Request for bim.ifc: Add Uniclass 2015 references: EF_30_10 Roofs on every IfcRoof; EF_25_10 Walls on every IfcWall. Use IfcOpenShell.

First a look at what the model holds.

```python
import ifcopenshell

model = ifcopenshell.open("bim.ifc")
print(model.schema)
print("classifications:", [c.Name for c in model.by_type("IfcClassification")])
for ifc_class in ("IfcDoor", "IfcRoof", "IfcStair", "IfcWall", "IfcWindow"):
    print(ifc_class, len(model.by_type(ifc_class)))
```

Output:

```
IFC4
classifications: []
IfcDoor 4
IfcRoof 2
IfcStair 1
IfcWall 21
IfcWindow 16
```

```python
import ifcopenshell
import ifcopenshell.api.classification

model = ifcopenshell.open("bim.ifc")

system = ifcopenshell.api.classification.add_classification(model, classification="Uniclass 2015")

codes = {
    "IfcRoof": ("EF_30_10", "Roofs"),
    "IfcWall": ("EF_25_10", "Walls"),
}
for ifc_class, (code, name) in codes.items():
    products = model.by_type(ifc_class)
    ifcopenshell.api.classification.add_reference(
        model, products=products, classification=system, identification=code, name=name
    )
    print(code, len(products))

model.write("bim_updated.ifc")
```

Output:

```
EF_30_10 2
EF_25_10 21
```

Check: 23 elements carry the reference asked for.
